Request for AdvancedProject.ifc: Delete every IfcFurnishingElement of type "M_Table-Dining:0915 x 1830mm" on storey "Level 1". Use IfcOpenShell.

First a look at what the model holds.

```python
import ifcopenshell
import ifcopenshell.util.element

model = ifcopenshell.open("AdvancedProject.ifc")
print(model.schema)
storey = next(s for s in model.by_type("IfcBuildingStorey") if s.Name == "Level 1")
furniture = [e for e in ifcopenshell.util.element.get_decomposition(storey) if e.is_a("IfcFurnishingElement")]
seen = {}
for e in furniture:
    element_type = ifcopenshell.util.element.get_type(e)
    name = element_type.Name if element_type not in (None, e) else None
    seen[name] = seen.get(name, 0) + 1
for name, count in sorted(seen.items(), key=str):
    print(count, "x", name)
```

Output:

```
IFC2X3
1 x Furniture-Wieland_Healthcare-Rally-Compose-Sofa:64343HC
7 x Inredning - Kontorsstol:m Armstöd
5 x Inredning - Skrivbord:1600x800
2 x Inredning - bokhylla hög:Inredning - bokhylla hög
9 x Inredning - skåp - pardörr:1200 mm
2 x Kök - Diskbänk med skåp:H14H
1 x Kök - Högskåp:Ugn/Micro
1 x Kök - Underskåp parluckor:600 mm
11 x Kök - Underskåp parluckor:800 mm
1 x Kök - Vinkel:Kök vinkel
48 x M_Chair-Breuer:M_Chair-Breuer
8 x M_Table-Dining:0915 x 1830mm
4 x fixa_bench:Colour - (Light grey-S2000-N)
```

```python
import ifcopenshell
import ifcopenshell.api.root
import ifcopenshell.util.element

model = ifcopenshell.open("AdvancedProject.ifc")

storey = next(s for s in model.by_type("IfcBuildingStorey") if s.Name == "Level 1")
furniture = [e for e in ifcopenshell.util.element.get_decomposition(storey) if e.is_a("IfcFurnishingElement")]
targets = [e for e in furniture if (t := ifcopenshell.util.element.get_type(e)) not in (None, e) and t.Name == "M_Table-Dining:0915 x 1830mm"]

for e in targets:
    ifcopenshell.api.root.remove_product(model, product=e)
print(len(targets), "removed")

model.write("AdvancedProject_edited.ifc")
```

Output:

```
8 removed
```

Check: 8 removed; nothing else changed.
